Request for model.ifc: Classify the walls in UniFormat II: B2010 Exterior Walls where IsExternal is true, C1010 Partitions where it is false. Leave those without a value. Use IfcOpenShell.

First a look at what the model holds.

```python
import ifcopenshell
import ifcopenshell.util.element

model = ifcopenshell.open("model.ifc")
print(model.schema)
print("classifications:", [c.Name for c in model.by_type("IfcClassification")])
values = [ifcopenshell.util.element.get_pset(e, "Pset_WallCommon", "IsExternal") for e in model.by_type("IfcWall")]
for value in (True, False, None):
    print("IsExternal", value, values.count(value))
```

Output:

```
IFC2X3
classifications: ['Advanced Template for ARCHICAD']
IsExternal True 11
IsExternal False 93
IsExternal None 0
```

```python
import ifcopenshell
import ifcopenshell.api.classification
import ifcopenshell.util.element

model = ifcopenshell.open("model.ifc")

# IFC2X3 requires Source and Edition and has no link from the project to the system.
system = model.create_entity("IfcClassification", Source="ASTM", Edition="E1557", Name="UniFormat II")

walls = model.by_type("IfcWall")
external = {e: ifcopenshell.util.element.get_pset(e, "Pset_WallCommon", "IsExternal") for e in walls}
for flag, code, name in ((True, "B2010", "Exterior Walls"), (False, "C1010", "Partitions")):
    products = [e for e in walls if external[e] is flag]
    ifcopenshell.api.classification.add_reference(
        model, products=products, classification=system, identification=code, name=name
    )
    print(code, len(products))

model.write("model_v2.ifc")
```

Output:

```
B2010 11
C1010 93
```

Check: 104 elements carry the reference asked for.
